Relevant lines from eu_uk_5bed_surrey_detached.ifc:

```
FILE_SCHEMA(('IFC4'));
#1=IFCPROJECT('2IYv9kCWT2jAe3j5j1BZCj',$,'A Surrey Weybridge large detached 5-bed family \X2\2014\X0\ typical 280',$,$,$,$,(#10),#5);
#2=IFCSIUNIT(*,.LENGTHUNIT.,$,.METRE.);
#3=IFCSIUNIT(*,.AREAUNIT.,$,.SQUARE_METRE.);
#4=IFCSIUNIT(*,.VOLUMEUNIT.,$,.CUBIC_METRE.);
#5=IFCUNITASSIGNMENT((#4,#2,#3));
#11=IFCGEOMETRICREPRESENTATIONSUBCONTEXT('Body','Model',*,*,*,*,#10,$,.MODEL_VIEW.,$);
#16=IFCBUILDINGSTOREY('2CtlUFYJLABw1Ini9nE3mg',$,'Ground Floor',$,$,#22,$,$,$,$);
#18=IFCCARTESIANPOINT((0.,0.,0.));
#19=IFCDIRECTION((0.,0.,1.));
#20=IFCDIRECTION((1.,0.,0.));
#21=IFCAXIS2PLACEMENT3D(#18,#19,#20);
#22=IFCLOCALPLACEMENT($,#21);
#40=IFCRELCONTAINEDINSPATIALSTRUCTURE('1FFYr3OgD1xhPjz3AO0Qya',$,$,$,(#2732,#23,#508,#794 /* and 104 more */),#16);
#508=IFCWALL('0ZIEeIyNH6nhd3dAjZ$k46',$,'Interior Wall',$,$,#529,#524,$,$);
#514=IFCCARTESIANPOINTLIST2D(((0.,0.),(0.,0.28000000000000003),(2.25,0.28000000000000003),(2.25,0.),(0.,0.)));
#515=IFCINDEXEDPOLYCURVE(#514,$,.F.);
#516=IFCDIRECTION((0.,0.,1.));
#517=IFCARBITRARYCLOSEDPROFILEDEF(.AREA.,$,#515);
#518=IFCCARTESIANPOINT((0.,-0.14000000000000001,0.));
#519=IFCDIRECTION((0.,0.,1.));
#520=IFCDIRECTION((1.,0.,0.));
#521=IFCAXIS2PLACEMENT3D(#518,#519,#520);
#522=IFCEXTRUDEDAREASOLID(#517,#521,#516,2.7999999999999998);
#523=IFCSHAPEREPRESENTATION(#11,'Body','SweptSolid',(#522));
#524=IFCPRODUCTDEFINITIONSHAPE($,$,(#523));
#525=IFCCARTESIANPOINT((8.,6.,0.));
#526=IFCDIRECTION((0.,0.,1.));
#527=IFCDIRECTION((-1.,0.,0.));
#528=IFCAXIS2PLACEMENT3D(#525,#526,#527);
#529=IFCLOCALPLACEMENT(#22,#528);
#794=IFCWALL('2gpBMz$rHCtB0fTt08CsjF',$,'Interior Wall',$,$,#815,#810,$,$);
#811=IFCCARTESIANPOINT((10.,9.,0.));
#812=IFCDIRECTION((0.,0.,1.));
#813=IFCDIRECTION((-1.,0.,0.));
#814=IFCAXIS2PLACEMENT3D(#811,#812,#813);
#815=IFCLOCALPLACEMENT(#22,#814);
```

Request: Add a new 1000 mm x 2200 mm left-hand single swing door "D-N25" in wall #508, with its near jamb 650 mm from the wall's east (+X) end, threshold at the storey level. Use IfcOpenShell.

```python
import numpy as np
import ifcopenshell
import ifcopenshell.api.feature
import ifcopenshell.api.geometry
import ifcopenshell.api.root
import ifcopenshell.api.spatial
import ifcopenshell.geom
import ifcopenshell.util.element
import ifcopenshell.util.placement
import ifcopenshell.util.representation
import ifcopenshell.util.shape
import ifcopenshell.util.unit

model = ifcopenshell.open("eu_uk_5bed_surrey_detached.ifc")
unit_scale = ifcopenshell.util.unit.calculate_unit_scale(model)
settings = ifcopenshell.geom.settings()


def volume(element):
    """Net volume in cubic metres, openings subtracted."""
    shape = ifcopenshell.geom.create_shape(settings, element)
    return ifcopenshell.util.shape.get_volume(shape.geometry)


wall = model.by_guid("0ZIEeIyNH6nhd3dAjZ$k46")
storey = ifcopenshell.util.element.get_container(wall, ifc_class="IfcBuildingStorey")
context = ifcopenshell.util.representation.get_context(model, "Model", "Body", "MODEL_VIEW")
before = volume(wall)

width, height, from_end, sill = 1, 2.2, 0.65, 0.0  # metres

# The wall runs along its own X axis, and the end named is its -X end.
wall_shape = ifcopenshell.geom.create_shape(settings, wall)
x, y, z = ifcopenshell.util.shape.get_vertices(wall_shape.geometry).T
start = x.min() + from_end
face, thickness = float(y.min()), float(y.max() - y.min())
wall_matrix = ifcopenshell.util.placement.get_local_placement(wall.ObjectPlacement)
level = ifcopenshell.util.placement.get_local_placement(storey.ObjectPlacement)[2, 3]


def in_wall(x, y):
    """Placement at x, y metres in the wall's axes, at sill height."""
    matrix = wall_matrix.copy()
    matrix[:, 3] = wall_matrix @ np.array([x / unit_scale, y / unit_scale, 0.0, 1.0])
    matrix[2, 3] = level + sill / unit_scale
    return matrix


# Opening: a box that overshoots both wall faces by 50 mm.
opening = ifcopenshell.api.root.create_entity(model, ifc_class="IfcOpeningElement", predefined_type="OPENING")
box = ifcopenshell.api.geometry.add_wall_representation(
    model, context=context, length=width, height=height, thickness=thickness + 0.1
)
ifcopenshell.api.geometry.assign_representation(model, product=opening, representation=box)
ifcopenshell.api.geometry.edit_object_placement(model, product=opening, matrix=in_wall(start, face - 0.05), is_si=False)
ifcopenshell.api.feature.add_feature(model, feature=opening, element=wall)

door = ifcopenshell.api.root.create_entity(model, ifc_class="IfcDoor", name="D-N25", predefined_type="DOOR")
door.OverallWidth, door.OverallHeight = width / unit_scale, height / unit_scale
door.OperationType = "SINGLE_SWING_LEFT"
body = ifcopenshell.api.geometry.add_door_representation(
    model,
    context=context,
    overall_width=door.OverallWidth,
    overall_height=door.OverallHeight,
    operation_type="SINGLE_SWING_LEFT",
    lining_properties={"LiningDepth": thickness / unit_scale, "ThresholdDepth": thickness / unit_scale},
)
ifcopenshell.api.geometry.assign_representation(model, product=door, representation=body)
ifcopenshell.api.spatial.assign_container(model, products=[door], relating_structure=storey)
ifcopenshell.api.feature.add_filling(model, opening=opening, element=door)

# The lining spans the wall, so the door starts at the wall face.
ifcopenshell.api.geometry.edit_object_placement(model, product=door, matrix=in_wall(start, face), is_si=False)

after = volume(wall)

print(f"wall volume {before:.3f} -> {after:.3f} m3")

model.write("eu_uk_5bed_surrey_detached_updated.ifc")
```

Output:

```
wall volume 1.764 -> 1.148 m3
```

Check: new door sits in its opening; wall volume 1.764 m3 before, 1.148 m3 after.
